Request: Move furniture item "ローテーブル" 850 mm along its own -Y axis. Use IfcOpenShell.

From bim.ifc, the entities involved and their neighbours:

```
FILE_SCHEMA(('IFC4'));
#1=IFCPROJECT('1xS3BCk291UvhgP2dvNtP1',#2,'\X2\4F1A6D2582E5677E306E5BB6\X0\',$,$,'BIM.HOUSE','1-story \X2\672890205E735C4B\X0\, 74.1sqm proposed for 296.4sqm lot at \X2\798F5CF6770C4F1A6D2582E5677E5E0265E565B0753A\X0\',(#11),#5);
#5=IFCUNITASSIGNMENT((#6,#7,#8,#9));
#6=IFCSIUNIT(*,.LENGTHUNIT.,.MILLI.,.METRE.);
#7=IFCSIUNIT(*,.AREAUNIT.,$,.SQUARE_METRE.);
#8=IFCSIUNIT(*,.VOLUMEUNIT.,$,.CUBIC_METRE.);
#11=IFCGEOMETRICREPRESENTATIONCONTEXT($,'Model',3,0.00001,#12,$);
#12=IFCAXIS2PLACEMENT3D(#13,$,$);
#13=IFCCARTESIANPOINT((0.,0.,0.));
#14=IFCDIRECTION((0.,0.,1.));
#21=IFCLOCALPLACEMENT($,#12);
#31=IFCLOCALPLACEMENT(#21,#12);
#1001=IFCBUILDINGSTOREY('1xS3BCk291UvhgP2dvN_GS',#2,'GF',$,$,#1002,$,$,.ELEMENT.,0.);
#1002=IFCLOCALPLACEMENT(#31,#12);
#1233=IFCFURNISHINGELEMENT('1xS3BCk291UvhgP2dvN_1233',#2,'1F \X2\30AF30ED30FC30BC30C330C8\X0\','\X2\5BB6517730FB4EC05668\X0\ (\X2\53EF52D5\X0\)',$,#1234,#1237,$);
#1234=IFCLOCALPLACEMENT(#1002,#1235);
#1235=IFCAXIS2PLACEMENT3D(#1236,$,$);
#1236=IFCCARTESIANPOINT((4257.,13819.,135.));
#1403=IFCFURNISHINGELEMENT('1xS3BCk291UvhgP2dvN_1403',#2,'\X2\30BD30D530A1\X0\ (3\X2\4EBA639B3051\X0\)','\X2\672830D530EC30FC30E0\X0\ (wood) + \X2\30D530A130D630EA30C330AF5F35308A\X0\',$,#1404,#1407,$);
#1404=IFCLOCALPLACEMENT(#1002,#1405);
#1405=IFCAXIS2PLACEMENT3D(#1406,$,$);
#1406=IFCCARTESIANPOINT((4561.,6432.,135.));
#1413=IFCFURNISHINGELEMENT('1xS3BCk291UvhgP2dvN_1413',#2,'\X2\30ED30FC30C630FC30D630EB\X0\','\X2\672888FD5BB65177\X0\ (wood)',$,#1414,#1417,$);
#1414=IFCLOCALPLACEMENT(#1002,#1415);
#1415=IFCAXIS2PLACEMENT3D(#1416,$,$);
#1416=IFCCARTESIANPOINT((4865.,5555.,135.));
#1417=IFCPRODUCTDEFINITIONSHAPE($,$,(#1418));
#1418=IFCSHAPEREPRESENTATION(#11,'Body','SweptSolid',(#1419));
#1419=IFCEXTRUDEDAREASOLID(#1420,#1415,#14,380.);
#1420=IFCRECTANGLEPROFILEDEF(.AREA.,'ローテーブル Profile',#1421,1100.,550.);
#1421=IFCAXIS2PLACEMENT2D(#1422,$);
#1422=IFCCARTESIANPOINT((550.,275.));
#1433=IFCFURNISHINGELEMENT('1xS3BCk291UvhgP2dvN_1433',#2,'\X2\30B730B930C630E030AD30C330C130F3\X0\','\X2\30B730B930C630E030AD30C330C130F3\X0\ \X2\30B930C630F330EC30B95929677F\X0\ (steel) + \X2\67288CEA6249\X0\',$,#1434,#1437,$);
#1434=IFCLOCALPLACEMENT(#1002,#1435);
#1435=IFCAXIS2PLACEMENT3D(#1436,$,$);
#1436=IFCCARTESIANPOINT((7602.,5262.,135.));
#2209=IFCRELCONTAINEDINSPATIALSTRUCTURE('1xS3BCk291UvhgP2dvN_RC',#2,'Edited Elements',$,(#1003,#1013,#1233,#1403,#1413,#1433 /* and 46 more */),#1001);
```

```python
import ifcopenshell
import ifcopenshell.api.geometry
import ifcopenshell.util.placement

model = ifcopenshell.open("bim.ifc")

item = model.by_guid("1xS3BCk291UvhgP2dvN_1413")
matrix = ifcopenshell.util.placement.get_local_placement(item.ObjectPlacement)
matrix[:3, 3] -= matrix[:3, 1] * 850.0
ifcopenshell.api.geometry.edit_object_placement(model, product=item, matrix=matrix, is_si=False)

print(ifcopenshell.util.placement.get_local_placement(item.ObjectPlacement).round(3) + 0.0)

model.write("bim_rev.ifc")
```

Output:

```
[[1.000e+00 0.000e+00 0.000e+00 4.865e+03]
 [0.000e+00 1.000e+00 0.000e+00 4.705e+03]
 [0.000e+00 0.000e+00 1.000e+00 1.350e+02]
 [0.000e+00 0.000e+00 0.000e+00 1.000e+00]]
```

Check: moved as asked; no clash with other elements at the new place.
